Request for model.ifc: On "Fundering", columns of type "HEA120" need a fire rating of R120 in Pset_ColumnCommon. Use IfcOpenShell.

First a look at what the model holds.

```python
import ifcopenshell
import ifcopenshell.util.element

model = ifcopenshell.open("model.ifc")
print(model.schema)
storey = next(s for s in model.by_type("IfcBuildingStorey") if s.Name == "Fundering")
columns = [e for e in ifcopenshell.util.element.get_decomposition(storey) if e.is_a("IfcColumn")]
seen = {}
for e in columns:
    element_type = ifcopenshell.util.element.get_type(e)
    key = (element_type.Name if element_type != e and element_type else None, ifcopenshell.util.element.get_pset(e, "Pset_ColumnCommon", "FireRating"))
    seen[key] = seen.get(key, 0) + 1
for (name, value), count in sorted(seen.items(), key=str):
    print(count, "x", name, "|", value)
```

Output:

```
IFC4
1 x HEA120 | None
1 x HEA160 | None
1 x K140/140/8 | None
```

```python
import ifcopenshell
import ifcopenshell.api.pset
import ifcopenshell.util.element

model = ifcopenshell.open("model.ifc")

storey = next(s for s in model.by_type("IfcBuildingStorey") if s.Name == "Fundering")
columns = [e for e in ifcopenshell.util.element.get_decomposition(storey) if e.is_a("IfcColumn")]

count = 0
for e in columns:
    element_type = ifcopenshell.util.element.get_type(e)
    if element_type in (None, e) or element_type.Name != "HEA120":
        continue
    # add_pset returns the element's existing set when there is one.
    pset = ifcopenshell.api.pset.add_pset(model, product=e, name="Pset_ColumnCommon")
    ifcopenshell.api.pset.edit_pset(model, pset=pset, properties={"FireRating": "R120"})
    count += 1

print(count, "columns updated")

model.write("model_rev.ifc")
```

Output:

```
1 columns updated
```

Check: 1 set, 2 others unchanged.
